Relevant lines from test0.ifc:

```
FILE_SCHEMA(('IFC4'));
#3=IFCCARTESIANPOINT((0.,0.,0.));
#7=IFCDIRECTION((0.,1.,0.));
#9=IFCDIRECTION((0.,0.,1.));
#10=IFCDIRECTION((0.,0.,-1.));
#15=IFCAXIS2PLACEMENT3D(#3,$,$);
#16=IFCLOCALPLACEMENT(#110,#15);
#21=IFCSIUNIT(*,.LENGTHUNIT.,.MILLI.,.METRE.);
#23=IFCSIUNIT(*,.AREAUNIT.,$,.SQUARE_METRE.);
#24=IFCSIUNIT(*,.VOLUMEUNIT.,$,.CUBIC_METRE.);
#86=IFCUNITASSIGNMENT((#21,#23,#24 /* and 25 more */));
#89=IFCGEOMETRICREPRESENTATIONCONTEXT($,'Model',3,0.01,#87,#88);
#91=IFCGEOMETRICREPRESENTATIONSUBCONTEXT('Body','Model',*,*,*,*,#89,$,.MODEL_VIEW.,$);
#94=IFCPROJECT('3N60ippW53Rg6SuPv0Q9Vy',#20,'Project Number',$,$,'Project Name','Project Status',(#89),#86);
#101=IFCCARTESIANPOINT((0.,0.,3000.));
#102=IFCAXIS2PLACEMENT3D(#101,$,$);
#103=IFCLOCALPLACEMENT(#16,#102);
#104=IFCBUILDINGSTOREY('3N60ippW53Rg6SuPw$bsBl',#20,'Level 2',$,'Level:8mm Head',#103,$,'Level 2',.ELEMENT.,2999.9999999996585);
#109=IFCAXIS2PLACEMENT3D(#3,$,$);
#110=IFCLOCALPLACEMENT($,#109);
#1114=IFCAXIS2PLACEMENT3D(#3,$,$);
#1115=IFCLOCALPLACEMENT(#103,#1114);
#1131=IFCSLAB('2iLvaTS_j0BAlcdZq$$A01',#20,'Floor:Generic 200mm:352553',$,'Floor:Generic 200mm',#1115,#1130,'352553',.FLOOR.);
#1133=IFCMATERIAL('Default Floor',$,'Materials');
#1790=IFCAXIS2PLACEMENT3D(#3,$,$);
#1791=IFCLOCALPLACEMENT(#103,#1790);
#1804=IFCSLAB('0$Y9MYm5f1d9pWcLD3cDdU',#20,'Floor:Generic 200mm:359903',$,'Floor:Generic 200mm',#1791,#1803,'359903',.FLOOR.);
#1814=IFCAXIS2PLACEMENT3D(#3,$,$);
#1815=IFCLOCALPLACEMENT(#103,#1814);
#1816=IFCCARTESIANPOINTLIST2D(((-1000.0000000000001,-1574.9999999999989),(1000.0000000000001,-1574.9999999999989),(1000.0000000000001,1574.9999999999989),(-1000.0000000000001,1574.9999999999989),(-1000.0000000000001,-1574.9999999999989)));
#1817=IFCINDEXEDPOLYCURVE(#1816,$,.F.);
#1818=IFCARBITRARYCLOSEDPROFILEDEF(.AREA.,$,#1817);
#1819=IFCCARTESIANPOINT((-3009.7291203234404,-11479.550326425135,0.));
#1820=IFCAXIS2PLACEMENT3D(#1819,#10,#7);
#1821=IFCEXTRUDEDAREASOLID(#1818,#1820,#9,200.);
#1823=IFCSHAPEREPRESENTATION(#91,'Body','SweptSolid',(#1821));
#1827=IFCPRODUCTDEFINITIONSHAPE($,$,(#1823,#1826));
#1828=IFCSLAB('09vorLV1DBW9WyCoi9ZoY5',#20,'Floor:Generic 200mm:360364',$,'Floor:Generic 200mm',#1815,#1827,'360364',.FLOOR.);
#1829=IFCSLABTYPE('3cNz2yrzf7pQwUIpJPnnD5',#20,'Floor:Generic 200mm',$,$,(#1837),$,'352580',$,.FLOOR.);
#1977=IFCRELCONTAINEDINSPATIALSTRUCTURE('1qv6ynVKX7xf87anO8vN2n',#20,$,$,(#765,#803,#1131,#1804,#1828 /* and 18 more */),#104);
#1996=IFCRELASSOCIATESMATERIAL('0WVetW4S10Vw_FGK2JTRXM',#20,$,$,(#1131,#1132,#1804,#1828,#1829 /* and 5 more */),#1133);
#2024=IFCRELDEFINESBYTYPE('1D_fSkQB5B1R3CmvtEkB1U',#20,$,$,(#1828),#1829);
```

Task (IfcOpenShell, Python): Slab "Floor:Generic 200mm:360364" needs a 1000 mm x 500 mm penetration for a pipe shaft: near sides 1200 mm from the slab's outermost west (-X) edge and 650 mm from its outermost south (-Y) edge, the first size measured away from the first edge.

```python
import numpy as np
import ifcopenshell
import ifcopenshell.api.feature
import ifcopenshell.api.geometry
import ifcopenshell.api.root
import ifcopenshell.geom
import ifcopenshell.util.placement
import ifcopenshell.util.representation
import ifcopenshell.util.shape
import ifcopenshell.util.unit

model = ifcopenshell.open("test0.ifc")
unit_scale = ifcopenshell.util.unit.calculate_unit_scale(model)
settings = ifcopenshell.geom.settings()


def volume(element):
    """Net volume in cubic metres, openings subtracted."""
    shape = ifcopenshell.geom.create_shape(settings, element)
    return ifcopenshell.util.shape.get_volume(shape.geometry)


slab = model.by_guid("09vorLV1DBW9WyCoi9ZoY5")
before = volume(slab)

# Extent in the slab's own axes, in metres. The edges named are its -X and -Y sides.
slab_shape = ifcopenshell.geom.create_shape(settings, slab)
vertices = ifcopenshell.util.shape.get_vertices(slab_shape.geometry)
x_min, y_min, bottom = vertices.min(axis=0)
top = vertices[:, 2].max()

opening = ifcopenshell.api.root.create_entity(model, ifc_class="IfcOpeningElement", name="Pipe shaft opening", predefined_type="OPENING")
context = ifcopenshell.util.representation.get_context(model, "Model", "Body", "MODEL_VIEW")
width, depth = 1, 0.5
outline = [(0.0, 0.0), (width, 0.0), (width, depth), (0.0, depth), (0.0, 0.0)]
# Overshoot both faces by 50 mm so the cut is clean.
shape = ifcopenshell.api.geometry.add_slab_representation(
    model, context=context, depth=top - bottom + 0.1, polyline=outline
)
ifcopenshell.api.geometry.assign_representation(model, product=opening, representation=shape)

matrix = ifcopenshell.util.placement.get_local_placement(slab.ObjectPlacement)
matrix[:, 3] = matrix @ np.append(np.array([x_min + 1.2, y_min + 0.65, bottom - 0.05]) / unit_scale, 1.0)
ifcopenshell.api.geometry.edit_object_placement(model, product=opening, matrix=matrix, is_si=False)
ifcopenshell.api.feature.add_feature(model, feature=opening, element=slab)

after = volume(slab)

print(f"slab volume {before:.3f} -> {after:.3f} m3")

model.write("test0_edited.ifc")
```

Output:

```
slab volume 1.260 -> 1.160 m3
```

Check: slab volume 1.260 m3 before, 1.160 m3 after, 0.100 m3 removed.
